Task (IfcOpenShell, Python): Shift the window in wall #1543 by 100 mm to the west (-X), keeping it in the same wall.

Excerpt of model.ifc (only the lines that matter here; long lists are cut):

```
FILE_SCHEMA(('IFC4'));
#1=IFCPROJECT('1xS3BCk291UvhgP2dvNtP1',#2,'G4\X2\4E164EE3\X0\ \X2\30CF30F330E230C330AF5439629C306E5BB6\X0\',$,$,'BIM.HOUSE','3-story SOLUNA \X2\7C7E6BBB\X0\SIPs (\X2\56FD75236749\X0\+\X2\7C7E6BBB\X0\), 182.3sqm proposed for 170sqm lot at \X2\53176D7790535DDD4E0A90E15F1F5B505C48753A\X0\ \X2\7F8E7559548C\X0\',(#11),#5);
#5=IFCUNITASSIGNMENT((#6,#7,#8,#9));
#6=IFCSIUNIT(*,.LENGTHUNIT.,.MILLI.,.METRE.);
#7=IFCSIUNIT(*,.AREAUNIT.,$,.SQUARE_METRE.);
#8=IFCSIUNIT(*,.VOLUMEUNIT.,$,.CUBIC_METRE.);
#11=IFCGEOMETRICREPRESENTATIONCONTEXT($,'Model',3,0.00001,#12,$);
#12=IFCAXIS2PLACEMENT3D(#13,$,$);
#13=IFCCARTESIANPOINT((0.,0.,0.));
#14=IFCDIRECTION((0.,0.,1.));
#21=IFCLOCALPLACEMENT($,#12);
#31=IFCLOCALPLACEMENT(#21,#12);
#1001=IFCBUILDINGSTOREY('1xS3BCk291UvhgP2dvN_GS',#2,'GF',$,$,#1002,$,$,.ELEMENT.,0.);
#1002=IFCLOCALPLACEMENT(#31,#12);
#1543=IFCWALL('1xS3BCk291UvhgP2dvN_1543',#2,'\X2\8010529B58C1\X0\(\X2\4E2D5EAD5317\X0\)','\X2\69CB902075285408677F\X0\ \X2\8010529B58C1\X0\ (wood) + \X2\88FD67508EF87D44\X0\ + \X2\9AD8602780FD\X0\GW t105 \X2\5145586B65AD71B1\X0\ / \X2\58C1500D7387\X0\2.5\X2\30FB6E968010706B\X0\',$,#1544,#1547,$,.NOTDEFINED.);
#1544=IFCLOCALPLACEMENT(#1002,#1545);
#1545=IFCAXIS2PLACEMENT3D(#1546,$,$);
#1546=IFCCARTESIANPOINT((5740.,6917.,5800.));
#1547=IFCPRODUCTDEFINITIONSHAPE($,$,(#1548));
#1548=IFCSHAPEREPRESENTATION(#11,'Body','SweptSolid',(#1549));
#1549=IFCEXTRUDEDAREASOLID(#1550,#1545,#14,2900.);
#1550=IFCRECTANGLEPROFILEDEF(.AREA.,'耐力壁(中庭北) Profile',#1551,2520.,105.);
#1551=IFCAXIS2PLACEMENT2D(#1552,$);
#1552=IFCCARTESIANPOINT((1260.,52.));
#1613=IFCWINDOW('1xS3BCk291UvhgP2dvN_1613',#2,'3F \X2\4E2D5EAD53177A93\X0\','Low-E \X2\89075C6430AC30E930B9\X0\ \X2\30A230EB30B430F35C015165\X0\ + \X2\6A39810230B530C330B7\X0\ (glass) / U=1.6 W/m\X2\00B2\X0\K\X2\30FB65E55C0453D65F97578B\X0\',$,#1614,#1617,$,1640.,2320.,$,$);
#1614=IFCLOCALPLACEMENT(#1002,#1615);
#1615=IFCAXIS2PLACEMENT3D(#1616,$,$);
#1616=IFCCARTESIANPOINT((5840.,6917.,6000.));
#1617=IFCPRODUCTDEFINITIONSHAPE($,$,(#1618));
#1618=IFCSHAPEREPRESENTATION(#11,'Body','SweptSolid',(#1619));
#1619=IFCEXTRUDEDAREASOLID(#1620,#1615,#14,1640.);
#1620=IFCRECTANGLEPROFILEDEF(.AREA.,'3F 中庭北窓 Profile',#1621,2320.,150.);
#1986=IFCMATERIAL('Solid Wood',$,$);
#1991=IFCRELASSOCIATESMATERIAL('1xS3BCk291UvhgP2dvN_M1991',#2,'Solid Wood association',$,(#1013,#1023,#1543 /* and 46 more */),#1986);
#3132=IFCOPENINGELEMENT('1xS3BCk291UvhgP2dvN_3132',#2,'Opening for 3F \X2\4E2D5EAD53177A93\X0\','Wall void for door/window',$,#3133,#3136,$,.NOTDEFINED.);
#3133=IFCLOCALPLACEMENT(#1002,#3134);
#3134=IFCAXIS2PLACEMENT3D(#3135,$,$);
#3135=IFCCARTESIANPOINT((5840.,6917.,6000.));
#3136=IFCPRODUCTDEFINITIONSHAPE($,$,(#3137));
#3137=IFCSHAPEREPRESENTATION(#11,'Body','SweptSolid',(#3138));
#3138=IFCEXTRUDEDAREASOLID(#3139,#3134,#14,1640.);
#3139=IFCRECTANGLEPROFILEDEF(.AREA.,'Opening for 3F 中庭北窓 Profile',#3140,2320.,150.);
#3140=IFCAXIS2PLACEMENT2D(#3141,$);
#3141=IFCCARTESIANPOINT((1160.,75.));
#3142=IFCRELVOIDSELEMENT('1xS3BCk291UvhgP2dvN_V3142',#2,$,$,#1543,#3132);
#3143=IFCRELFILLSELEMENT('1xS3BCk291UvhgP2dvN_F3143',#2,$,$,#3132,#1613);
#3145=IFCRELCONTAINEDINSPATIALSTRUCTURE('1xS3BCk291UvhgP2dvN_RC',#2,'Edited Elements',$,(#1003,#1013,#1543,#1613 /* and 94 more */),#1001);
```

```python
import ifcopenshell
import ifcopenshell.api.geometry
import ifcopenshell.util.placement

model = ifcopenshell.open("model.ifc")

window = model.by_guid("1xS3BCk291UvhgP2dvN_1613")
opening = window.FillsVoids[0].RelatingOpeningElement
wall = opening.VoidsElements[0].RelatingBuildingElement

wall_matrix = ifcopenshell.util.placement.get_local_placement(wall.ObjectPlacement)
shift = wall_matrix[:3, 0] * -100.0
before = ifcopenshell.util.placement.get_local_placement(window.ObjectPlacement)[:3, 3].copy()

# The window is not placed relative to its opening, so move both.
for product in (opening, window):
    matrix = ifcopenshell.util.placement.get_local_placement(product.ObjectPlacement)
    matrix[:3, 3] += shift
    ifcopenshell.api.geometry.edit_object_placement(model, product=product, matrix=matrix, is_si=False)

after = ifcopenshell.util.placement.get_local_placement(window.ObjectPlacement)[:3, 3]
print("window moved by", (after - before).round(3) + 0.0)

model.write("model_rev.ifc")
```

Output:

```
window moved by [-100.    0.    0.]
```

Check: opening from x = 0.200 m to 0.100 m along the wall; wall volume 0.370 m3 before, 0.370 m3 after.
